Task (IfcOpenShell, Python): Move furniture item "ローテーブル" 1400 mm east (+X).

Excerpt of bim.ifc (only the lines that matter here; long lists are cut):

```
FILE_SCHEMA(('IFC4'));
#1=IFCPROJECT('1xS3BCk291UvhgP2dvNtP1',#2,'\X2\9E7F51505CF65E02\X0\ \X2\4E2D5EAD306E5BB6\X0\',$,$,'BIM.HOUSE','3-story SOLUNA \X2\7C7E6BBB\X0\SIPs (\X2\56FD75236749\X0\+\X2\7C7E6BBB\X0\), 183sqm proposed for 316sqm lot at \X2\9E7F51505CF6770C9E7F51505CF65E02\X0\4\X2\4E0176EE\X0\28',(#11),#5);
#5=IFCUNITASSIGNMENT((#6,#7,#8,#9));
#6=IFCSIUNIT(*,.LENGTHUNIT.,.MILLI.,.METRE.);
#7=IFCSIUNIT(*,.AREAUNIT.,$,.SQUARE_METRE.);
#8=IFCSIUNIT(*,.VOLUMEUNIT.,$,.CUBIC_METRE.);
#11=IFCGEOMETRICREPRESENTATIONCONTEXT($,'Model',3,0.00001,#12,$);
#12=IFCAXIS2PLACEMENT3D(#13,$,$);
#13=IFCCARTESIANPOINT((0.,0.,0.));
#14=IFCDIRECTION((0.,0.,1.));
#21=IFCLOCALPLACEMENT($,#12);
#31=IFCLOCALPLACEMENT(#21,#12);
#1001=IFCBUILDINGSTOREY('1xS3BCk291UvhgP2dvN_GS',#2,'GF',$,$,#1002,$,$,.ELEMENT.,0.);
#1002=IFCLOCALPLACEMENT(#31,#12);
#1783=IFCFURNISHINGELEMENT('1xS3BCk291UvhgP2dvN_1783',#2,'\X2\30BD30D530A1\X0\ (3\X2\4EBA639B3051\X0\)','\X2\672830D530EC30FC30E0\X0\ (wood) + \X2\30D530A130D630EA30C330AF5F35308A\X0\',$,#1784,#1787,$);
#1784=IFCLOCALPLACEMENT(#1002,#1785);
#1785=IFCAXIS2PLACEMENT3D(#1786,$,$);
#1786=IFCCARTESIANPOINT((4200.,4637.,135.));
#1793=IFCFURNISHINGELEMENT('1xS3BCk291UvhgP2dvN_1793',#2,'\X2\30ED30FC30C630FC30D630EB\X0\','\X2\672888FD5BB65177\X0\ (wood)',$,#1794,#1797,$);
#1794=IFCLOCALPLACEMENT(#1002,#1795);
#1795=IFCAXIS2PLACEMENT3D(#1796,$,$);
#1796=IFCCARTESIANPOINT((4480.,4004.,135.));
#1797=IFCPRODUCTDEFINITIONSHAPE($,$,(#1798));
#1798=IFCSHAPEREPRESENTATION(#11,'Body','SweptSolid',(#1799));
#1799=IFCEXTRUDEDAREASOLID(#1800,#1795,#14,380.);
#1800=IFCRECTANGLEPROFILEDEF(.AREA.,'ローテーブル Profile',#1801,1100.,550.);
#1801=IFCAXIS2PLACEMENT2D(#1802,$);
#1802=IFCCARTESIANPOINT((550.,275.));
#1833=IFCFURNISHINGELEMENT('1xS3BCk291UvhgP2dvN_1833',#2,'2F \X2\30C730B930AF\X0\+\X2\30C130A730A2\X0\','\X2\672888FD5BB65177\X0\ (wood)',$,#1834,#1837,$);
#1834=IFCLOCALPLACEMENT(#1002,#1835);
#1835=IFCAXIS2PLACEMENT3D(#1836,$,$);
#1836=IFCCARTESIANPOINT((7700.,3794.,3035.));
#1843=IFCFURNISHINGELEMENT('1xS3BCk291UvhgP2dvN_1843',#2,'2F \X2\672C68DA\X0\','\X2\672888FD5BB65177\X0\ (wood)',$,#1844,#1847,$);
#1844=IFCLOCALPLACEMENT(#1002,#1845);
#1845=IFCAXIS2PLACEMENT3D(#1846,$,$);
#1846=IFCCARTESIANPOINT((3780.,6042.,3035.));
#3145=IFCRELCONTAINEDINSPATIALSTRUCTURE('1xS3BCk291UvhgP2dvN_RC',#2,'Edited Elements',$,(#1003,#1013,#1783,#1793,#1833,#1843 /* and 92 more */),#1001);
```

```python
import ifcopenshell
import ifcopenshell.api.geometry
import ifcopenshell.util.placement
import ifcopenshell.util.unit

model = ifcopenshell.open("bim.ifc")
unit_scale = ifcopenshell.util.unit.calculate_unit_scale(model)

item = model.by_guid("1xS3BCk291UvhgP2dvN_1793")
matrix = ifcopenshell.util.placement.get_local_placement(item.ObjectPlacement)
matrix[0, 3] += 1.4 / unit_scale
ifcopenshell.api.geometry.edit_object_placement(model, product=item, matrix=matrix, is_si=False)

print(ifcopenshell.util.placement.get_local_placement(item.ObjectPlacement).round(3) + 0.0)

model.write("bim_v2.ifc")
```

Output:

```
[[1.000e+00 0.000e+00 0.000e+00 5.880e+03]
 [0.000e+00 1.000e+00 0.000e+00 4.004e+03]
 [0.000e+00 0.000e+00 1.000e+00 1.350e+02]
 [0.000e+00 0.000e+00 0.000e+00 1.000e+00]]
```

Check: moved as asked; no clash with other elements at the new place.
